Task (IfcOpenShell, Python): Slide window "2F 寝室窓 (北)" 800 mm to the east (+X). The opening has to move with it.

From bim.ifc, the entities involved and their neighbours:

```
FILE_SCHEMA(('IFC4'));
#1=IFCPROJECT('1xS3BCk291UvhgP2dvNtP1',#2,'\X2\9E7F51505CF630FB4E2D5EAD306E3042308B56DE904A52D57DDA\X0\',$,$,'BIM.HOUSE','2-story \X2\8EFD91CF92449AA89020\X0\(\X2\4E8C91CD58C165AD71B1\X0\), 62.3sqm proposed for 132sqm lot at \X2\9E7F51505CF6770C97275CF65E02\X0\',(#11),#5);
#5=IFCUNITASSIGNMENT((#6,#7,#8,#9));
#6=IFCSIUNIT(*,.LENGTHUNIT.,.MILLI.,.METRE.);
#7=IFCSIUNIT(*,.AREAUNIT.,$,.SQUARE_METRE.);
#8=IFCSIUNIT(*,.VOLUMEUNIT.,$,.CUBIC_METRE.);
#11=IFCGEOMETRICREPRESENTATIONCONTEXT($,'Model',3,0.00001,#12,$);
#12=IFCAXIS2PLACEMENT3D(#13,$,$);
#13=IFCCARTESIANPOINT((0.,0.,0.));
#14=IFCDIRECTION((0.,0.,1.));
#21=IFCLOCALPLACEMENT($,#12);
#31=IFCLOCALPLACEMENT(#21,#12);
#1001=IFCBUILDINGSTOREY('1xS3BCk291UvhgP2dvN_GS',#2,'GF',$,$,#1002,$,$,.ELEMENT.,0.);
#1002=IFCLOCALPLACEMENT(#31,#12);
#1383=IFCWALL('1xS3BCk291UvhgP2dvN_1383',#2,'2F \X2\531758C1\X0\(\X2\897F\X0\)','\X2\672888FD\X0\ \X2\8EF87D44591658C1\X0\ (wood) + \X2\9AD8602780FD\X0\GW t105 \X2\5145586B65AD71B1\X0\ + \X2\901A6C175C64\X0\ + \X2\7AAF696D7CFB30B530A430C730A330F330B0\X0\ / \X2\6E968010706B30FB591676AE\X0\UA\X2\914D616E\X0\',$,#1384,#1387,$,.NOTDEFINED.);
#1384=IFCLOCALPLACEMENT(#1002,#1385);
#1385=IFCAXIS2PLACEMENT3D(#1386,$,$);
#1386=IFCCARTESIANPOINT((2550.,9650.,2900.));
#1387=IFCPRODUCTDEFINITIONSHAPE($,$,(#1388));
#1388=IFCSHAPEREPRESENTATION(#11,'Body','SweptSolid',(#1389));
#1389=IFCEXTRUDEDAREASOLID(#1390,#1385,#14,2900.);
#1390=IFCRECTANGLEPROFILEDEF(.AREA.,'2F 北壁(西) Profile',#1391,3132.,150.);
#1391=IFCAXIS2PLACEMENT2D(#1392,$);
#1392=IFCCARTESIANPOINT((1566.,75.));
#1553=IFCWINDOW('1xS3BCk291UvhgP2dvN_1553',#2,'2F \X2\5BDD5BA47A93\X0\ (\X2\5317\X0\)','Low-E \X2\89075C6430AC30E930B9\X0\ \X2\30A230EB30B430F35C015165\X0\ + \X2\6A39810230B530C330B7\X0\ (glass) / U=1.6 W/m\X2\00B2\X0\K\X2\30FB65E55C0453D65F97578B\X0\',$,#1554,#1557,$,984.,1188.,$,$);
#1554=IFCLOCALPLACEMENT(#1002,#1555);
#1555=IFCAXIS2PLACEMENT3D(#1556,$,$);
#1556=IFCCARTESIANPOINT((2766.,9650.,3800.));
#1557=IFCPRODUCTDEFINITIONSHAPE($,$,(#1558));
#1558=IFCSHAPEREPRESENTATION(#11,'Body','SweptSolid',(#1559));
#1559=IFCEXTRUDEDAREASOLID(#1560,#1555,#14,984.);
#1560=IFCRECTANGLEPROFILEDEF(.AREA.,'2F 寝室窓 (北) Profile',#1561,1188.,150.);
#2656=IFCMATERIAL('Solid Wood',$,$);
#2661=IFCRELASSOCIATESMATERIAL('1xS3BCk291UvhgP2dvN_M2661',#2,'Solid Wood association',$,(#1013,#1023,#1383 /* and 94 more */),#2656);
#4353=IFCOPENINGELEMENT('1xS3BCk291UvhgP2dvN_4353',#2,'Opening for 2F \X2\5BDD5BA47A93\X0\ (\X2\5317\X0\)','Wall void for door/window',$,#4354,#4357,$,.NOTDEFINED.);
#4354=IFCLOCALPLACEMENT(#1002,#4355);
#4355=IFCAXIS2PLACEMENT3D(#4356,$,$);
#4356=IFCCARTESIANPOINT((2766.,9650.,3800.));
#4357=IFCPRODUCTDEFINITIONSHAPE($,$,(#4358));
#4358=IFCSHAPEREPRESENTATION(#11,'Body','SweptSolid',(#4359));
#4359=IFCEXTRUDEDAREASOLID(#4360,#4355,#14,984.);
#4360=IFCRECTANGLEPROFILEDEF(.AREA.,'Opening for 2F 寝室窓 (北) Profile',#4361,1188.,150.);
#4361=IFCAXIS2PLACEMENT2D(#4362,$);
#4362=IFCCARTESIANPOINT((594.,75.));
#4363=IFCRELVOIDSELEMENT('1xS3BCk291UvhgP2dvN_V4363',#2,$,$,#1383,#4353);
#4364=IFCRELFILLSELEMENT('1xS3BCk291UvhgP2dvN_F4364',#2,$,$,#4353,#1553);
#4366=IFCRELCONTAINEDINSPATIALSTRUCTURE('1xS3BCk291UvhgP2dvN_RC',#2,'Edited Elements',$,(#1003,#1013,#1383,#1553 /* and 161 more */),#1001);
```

```python
import ifcopenshell
import ifcopenshell.api.geometry
import ifcopenshell.util.placement

model = ifcopenshell.open("bim.ifc")

window = model.by_guid("1xS3BCk291UvhgP2dvN_1553")
opening = window.FillsVoids[0].RelatingOpeningElement
wall = opening.VoidsElements[0].RelatingBuildingElement

wall_matrix = ifcopenshell.util.placement.get_local_placement(wall.ObjectPlacement)
shift = wall_matrix[:3, 0] * 800.0
before = ifcopenshell.util.placement.get_local_placement(window.ObjectPlacement)[:3, 3].copy()

# The window is not placed relative to its opening, so move both.
for product in (opening, window):
    matrix = ifcopenshell.util.placement.get_local_placement(product.ObjectPlacement)
    matrix[:3, 3] += shift
    ifcopenshell.api.geometry.edit_object_placement(model, product=product, matrix=matrix, is_si=False)

after = ifcopenshell.util.placement.get_local_placement(window.ObjectPlacement)[:3, 3]
print("window moved by", (after - before).round(3) + 0.0)

model.write("bim_rev.ifc")
```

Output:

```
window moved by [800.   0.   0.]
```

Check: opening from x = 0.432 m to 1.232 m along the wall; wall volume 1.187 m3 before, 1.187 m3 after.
